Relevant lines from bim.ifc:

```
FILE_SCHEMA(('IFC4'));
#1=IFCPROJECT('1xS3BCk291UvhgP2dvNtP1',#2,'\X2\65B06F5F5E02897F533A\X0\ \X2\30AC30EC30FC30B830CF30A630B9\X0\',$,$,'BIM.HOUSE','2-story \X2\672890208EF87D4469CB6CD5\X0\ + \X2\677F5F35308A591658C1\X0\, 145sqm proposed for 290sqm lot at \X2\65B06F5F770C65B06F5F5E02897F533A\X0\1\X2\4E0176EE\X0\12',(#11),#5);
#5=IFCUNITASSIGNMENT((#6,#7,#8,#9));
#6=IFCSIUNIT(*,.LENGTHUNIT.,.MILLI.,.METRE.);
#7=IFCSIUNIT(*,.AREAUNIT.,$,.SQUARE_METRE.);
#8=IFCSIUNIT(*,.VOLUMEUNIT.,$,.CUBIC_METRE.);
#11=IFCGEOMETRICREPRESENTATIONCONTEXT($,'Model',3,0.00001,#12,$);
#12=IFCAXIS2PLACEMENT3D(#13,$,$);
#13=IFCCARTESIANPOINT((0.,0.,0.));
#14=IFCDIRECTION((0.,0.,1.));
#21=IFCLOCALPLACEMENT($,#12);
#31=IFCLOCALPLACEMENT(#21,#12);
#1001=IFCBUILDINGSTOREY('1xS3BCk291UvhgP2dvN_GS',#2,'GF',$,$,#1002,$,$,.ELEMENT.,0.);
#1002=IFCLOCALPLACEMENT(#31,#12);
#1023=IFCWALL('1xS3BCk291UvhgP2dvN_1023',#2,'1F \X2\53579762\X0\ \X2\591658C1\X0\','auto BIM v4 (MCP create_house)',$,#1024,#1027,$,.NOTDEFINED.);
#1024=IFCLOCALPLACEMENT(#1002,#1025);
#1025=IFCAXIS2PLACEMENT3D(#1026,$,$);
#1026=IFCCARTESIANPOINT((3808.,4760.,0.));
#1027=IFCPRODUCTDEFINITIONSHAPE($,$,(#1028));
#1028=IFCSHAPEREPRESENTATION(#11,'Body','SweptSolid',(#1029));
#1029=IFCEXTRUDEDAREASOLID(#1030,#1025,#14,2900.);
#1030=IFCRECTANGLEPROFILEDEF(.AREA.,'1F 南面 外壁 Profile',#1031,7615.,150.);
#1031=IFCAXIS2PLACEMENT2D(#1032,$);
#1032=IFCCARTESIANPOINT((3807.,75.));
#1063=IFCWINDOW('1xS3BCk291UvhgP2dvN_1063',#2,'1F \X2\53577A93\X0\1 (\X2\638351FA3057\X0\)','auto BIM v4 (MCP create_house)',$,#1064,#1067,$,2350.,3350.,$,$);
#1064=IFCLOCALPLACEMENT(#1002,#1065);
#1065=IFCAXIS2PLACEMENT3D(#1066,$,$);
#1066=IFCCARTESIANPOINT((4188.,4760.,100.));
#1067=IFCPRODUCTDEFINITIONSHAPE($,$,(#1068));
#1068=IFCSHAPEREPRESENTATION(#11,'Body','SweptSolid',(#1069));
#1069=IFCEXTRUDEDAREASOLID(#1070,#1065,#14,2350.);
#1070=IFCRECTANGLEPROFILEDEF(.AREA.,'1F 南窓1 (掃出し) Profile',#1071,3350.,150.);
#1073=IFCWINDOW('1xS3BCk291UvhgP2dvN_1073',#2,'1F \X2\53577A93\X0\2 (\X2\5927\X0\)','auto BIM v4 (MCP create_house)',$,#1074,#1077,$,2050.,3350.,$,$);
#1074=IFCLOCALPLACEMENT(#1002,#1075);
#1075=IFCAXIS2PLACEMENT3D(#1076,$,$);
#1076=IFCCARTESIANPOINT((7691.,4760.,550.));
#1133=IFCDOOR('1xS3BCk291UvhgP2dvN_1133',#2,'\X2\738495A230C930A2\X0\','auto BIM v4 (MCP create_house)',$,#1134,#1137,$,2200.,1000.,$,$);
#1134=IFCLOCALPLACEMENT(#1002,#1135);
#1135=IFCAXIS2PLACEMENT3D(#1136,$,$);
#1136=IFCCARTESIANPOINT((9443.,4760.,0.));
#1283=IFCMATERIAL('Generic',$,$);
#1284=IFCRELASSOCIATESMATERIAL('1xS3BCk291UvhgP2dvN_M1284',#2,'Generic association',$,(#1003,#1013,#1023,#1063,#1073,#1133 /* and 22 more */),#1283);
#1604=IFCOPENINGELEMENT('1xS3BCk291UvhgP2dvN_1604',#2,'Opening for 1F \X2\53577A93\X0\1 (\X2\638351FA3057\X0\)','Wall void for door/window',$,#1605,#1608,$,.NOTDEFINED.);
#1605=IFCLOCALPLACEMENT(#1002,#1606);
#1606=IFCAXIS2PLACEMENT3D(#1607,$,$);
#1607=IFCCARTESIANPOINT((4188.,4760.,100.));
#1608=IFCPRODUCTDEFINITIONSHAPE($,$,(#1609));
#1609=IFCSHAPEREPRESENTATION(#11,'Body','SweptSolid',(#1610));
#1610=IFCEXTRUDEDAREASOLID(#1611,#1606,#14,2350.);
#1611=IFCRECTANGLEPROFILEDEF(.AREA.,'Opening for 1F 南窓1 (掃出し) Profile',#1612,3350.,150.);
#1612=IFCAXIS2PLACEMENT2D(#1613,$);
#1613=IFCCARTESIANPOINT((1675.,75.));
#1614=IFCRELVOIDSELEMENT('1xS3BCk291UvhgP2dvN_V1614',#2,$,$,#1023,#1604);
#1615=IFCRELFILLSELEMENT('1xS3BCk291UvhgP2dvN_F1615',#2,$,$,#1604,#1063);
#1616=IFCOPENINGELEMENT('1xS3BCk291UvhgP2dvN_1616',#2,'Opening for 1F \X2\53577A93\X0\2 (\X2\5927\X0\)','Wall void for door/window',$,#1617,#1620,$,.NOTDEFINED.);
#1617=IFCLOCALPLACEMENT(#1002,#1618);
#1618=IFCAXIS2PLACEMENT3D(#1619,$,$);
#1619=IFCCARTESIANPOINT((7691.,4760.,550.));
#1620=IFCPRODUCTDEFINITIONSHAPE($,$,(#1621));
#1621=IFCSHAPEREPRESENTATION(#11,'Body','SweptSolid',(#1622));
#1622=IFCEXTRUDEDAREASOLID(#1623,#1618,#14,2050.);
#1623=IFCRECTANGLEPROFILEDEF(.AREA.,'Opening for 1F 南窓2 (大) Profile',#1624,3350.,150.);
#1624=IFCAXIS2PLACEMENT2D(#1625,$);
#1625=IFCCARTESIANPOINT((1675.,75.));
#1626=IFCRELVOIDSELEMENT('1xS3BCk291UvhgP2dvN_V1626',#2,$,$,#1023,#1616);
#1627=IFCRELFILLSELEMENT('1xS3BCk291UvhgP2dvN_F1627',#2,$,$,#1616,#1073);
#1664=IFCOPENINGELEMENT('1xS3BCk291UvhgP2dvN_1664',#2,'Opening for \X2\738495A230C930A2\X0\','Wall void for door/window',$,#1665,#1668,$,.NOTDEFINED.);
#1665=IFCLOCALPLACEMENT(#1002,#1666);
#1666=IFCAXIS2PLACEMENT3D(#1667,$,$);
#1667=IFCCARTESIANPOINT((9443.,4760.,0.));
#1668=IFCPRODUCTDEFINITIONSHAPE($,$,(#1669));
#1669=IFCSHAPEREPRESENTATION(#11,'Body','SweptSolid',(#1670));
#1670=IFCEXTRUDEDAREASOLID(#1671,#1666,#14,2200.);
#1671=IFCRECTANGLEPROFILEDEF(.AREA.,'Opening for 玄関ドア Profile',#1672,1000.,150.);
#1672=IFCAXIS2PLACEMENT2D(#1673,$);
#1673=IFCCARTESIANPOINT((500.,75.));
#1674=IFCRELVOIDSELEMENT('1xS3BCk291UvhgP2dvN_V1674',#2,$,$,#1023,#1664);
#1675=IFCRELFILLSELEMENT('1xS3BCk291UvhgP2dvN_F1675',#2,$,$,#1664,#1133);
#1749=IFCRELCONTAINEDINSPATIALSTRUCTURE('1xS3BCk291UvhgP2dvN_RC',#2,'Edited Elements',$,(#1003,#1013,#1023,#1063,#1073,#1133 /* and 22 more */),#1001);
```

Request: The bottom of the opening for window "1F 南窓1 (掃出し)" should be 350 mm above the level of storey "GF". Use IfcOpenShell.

```python
import numpy as np
import ifcopenshell
import ifcopenshell.api.geometry
import ifcopenshell.geom
import ifcopenshell.util.element
import ifcopenshell.util.placement
import ifcopenshell.util.shape
import ifcopenshell.util.unit

model = ifcopenshell.open("bim.ifc")
unit_scale = ifcopenshell.util.unit.calculate_unit_scale(model)

window = model.by_guid("1xS3BCk291UvhgP2dvN_1063")
opening = window.FillsVoids[0].RelatingOpeningElement
storey = ifcopenshell.util.element.get_container(window, ifc_class="IfcBuildingStorey")
level = ifcopenshell.util.placement.get_local_placement(storey.ObjectPlacement)[2, 3]

# The opening's origin need not be at the sill, so measure its lowest point.
shape = ifcopenshell.geom.create_shape(ifcopenshell.geom.settings(), opening)
bottom = ifcopenshell.util.shape.get_shape_bottom_elevation(shape, shape.geometry) / unit_scale
dz = level + 0.35 / unit_scale - bottom

shift = np.array([0.0, 0.0, dz])
# The window is not placed relative to its opening, so move both.
for product in (opening, window):
    matrix = ifcopenshell.util.placement.get_local_placement(product.ObjectPlacement)
    matrix[:3, 3] += shift
    ifcopenshell.api.geometry.edit_object_placement(model, product=product, matrix=matrix, is_si=False)

print(f"moved by {dz * unit_scale:+.3f} m")

model.write("bim_edited.ifc")
```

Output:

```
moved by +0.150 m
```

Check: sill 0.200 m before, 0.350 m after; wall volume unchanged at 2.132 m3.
